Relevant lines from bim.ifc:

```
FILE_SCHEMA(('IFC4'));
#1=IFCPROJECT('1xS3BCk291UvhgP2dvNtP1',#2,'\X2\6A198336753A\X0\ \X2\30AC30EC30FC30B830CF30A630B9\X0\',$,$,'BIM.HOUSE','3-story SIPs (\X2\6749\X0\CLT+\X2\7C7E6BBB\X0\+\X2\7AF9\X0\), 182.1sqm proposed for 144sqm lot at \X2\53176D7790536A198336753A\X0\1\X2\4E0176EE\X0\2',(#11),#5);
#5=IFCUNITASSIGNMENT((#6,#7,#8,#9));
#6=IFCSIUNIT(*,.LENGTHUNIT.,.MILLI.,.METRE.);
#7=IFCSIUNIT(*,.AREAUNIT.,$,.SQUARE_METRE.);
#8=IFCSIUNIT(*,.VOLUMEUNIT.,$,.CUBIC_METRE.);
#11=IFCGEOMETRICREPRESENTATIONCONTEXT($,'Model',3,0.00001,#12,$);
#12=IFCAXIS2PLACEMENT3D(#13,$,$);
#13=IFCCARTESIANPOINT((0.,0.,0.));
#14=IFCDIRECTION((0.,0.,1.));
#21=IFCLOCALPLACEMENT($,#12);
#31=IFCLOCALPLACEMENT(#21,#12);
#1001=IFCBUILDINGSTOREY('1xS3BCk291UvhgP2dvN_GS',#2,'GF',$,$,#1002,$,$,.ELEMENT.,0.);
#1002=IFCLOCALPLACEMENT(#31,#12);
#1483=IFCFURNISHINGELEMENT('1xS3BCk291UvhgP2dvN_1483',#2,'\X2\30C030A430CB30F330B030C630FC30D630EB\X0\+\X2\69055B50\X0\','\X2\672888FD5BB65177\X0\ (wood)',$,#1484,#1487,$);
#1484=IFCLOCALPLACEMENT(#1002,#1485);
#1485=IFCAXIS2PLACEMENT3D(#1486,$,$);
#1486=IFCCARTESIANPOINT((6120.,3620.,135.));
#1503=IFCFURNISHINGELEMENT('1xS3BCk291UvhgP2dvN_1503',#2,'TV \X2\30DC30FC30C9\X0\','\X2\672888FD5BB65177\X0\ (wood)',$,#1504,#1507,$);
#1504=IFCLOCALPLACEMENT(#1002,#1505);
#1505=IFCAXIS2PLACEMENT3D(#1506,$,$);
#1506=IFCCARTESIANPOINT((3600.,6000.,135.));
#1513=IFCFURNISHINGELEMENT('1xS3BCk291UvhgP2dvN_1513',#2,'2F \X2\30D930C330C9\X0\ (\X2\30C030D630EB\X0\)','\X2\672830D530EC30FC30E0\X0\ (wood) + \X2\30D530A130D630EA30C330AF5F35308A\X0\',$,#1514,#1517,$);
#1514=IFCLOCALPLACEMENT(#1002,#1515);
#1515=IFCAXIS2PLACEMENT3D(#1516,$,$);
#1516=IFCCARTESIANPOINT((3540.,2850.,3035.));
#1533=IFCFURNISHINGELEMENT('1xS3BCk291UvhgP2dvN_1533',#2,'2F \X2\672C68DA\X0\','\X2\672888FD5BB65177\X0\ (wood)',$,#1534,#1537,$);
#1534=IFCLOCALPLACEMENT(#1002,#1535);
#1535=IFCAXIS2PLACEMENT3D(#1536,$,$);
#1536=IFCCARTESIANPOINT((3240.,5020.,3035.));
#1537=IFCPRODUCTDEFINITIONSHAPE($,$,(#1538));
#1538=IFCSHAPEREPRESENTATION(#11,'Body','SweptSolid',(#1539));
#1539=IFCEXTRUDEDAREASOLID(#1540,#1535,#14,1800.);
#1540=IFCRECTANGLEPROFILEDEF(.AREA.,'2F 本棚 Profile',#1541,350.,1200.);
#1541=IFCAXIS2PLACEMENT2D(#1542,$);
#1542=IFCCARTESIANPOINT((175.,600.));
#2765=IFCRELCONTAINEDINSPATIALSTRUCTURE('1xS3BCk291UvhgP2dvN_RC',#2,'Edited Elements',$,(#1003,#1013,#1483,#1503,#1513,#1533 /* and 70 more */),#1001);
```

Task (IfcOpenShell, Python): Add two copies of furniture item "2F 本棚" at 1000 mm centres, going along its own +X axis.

```python
import ifcopenshell
import ifcopenshell.api.geometry
import ifcopenshell.api.root
import ifcopenshell.util.element
import ifcopenshell.util.placement

model = ifcopenshell.open("bim.ifc")


def reuse_history(source, copy):
    """copy_class also copies each property set's owner history, people and application; keep the originals."""
    for rel in copy.IsDefinedBy:
        if rel.is_a("IfcRelDefinesByProperties") and (history := rel.RelatingPropertyDefinition.OwnerHistory):
            rel.RelatingPropertyDefinition.OwnerHistory = source.OwnerHistory
            ifcopenshell.util.element.remove_deep2(model, history)


source = model.by_guid("1xS3BCk291UvhgP2dvN_1533")
base = ifcopenshell.util.placement.get_local_placement(source.ObjectPlacement)
step = base[:3, 0] * 1000.0

for i in range(1, 3):
    copy = ifcopenshell.api.root.copy_class(model, product=source)
    copy.Representation = ifcopenshell.util.element.copy_deep(
        model, source.Representation, exclude=["IfcGeometricRepresentationContext", "IfcRepresentationMap"]
    )
    reuse_history(source, copy)
    matrix = base.copy()
    matrix[:3, 3] += i * step
    print("added at", matrix[:3, 3].round(3) + 0.0)
    ifcopenshell.api.geometry.edit_object_placement(model, product=copy, matrix=matrix, is_si=False)

model.write("bim_edited.ifc")
```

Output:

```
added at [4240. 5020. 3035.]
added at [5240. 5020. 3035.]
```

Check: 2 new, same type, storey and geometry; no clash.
